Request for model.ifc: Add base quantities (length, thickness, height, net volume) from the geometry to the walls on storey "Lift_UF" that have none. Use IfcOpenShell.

First a look at what the model holds.

```python
import ifcopenshell
import ifcopenshell.util.element
import ifcopenshell.util.unit

model = ifcopenshell.open("model.ifc")
print(model.schema)
for unit_type in ("LENGTHUNIT", "AREAUNIT", "VOLUMEUNIT"):
    print(unit_type, ifcopenshell.util.unit.calculate_unit_scale(model, unit_type))
storey = next(s for s in model.by_type("IfcBuildingStorey") if s.Name == "Lift_UF")
walls = [e for e in ifcopenshell.util.element.get_decomposition(storey) if e.is_a("IfcWall")]
for e in sorted(walls, key=lambda e: e.id()):
    print(e.id(), e.is_a(), e.Name, list(ifcopenshell.util.element.get_psets(e, qtos_only=True)), sep=" | ")
```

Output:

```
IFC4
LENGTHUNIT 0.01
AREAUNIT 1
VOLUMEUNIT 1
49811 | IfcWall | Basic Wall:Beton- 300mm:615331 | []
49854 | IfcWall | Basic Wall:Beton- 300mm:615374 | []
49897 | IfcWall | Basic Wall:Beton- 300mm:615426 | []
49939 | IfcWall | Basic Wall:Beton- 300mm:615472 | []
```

```python
import ifcopenshell
import ifcopenshell.api.pset
import ifcopenshell.geom
import ifcopenshell.util.element
import ifcopenshell.util.shape
import ifcopenshell.util.unit

model = ifcopenshell.open("model.ifc")
unit_scale = ifcopenshell.util.unit.calculate_unit_scale(model)
volume_scale = ifcopenshell.util.unit.calculate_unit_scale(model, "VOLUMEUNIT")
settings = ifcopenshell.geom.settings()

storey = next(s for s in model.by_type("IfcBuildingStorey") if s.Name == "Lift_UF")
walls = [e for e in ifcopenshell.util.element.get_decomposition(storey) if e.is_a("IfcWall")]

for e in sorted(walls, key=lambda e: e.id()):
    if ifcopenshell.util.element.get_psets(e, qtos_only=True, should_inherit=False):
        continue
    # Geometry comes back in metres, in the element's own axes.
    shape = ifcopenshell.geom.create_shape(settings, e)
    values = {
        "Length": ifcopenshell.util.shape.get_x(shape.geometry) / unit_scale,
        "Width": ifcopenshell.util.shape.get_y(shape.geometry) / unit_scale,
        "Height": ifcopenshell.util.shape.get_z(shape.geometry) / unit_scale,
        "NetVolume": ifcopenshell.util.shape.get_volume(shape.geometry) / volume_scale,
    }
    qto = ifcopenshell.api.pset.add_qto(model, product=e, name="Qto_WallBaseQuantities")
    ifcopenshell.api.pset.edit_qto(model, qto=qto, properties=values)
    print(e.id(), {k: round(v, 3) for k, v in values.items()})

model.write("model_v2.ifc")
```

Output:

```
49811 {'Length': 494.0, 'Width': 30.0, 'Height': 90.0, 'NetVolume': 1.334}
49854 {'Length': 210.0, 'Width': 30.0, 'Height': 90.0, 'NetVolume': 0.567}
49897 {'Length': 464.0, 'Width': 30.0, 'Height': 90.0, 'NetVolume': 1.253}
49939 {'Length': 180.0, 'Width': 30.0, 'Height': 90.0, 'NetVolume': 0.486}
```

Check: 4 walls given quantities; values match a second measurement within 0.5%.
